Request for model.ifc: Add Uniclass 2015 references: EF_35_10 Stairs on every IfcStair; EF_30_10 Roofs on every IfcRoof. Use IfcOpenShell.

First a look at what the model holds.

```python
import ifcopenshell

model = ifcopenshell.open("model.ifc")
print(model.schema)
print("classifications:", [c.Name for c in model.by_type("IfcClassification")])
for ifc_class in ("IfcDoor", "IfcRoof", "IfcStair", "IfcWall", "IfcWindow"):
    print(ifc_class, len(model.by_type(ifc_class)))
```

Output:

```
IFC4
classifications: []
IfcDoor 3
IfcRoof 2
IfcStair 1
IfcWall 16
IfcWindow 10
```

```python
import ifcopenshell
import ifcopenshell.api.classification

model = ifcopenshell.open("model.ifc")

system = ifcopenshell.api.classification.add_classification(model, classification="Uniclass 2015")

codes = {
    "IfcStair": ("EF_35_10", "Stairs"),
    "IfcRoof": ("EF_30_10", "Roofs"),
}
for ifc_class, (code, name) in codes.items():
    products = model.by_type(ifc_class)
    ifcopenshell.api.classification.add_reference(
        model, products=products, classification=system, identification=code, name=name
    )
    print(code, len(products))

model.write("model_v2.ifc")
```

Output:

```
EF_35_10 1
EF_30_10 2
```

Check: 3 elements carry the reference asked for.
